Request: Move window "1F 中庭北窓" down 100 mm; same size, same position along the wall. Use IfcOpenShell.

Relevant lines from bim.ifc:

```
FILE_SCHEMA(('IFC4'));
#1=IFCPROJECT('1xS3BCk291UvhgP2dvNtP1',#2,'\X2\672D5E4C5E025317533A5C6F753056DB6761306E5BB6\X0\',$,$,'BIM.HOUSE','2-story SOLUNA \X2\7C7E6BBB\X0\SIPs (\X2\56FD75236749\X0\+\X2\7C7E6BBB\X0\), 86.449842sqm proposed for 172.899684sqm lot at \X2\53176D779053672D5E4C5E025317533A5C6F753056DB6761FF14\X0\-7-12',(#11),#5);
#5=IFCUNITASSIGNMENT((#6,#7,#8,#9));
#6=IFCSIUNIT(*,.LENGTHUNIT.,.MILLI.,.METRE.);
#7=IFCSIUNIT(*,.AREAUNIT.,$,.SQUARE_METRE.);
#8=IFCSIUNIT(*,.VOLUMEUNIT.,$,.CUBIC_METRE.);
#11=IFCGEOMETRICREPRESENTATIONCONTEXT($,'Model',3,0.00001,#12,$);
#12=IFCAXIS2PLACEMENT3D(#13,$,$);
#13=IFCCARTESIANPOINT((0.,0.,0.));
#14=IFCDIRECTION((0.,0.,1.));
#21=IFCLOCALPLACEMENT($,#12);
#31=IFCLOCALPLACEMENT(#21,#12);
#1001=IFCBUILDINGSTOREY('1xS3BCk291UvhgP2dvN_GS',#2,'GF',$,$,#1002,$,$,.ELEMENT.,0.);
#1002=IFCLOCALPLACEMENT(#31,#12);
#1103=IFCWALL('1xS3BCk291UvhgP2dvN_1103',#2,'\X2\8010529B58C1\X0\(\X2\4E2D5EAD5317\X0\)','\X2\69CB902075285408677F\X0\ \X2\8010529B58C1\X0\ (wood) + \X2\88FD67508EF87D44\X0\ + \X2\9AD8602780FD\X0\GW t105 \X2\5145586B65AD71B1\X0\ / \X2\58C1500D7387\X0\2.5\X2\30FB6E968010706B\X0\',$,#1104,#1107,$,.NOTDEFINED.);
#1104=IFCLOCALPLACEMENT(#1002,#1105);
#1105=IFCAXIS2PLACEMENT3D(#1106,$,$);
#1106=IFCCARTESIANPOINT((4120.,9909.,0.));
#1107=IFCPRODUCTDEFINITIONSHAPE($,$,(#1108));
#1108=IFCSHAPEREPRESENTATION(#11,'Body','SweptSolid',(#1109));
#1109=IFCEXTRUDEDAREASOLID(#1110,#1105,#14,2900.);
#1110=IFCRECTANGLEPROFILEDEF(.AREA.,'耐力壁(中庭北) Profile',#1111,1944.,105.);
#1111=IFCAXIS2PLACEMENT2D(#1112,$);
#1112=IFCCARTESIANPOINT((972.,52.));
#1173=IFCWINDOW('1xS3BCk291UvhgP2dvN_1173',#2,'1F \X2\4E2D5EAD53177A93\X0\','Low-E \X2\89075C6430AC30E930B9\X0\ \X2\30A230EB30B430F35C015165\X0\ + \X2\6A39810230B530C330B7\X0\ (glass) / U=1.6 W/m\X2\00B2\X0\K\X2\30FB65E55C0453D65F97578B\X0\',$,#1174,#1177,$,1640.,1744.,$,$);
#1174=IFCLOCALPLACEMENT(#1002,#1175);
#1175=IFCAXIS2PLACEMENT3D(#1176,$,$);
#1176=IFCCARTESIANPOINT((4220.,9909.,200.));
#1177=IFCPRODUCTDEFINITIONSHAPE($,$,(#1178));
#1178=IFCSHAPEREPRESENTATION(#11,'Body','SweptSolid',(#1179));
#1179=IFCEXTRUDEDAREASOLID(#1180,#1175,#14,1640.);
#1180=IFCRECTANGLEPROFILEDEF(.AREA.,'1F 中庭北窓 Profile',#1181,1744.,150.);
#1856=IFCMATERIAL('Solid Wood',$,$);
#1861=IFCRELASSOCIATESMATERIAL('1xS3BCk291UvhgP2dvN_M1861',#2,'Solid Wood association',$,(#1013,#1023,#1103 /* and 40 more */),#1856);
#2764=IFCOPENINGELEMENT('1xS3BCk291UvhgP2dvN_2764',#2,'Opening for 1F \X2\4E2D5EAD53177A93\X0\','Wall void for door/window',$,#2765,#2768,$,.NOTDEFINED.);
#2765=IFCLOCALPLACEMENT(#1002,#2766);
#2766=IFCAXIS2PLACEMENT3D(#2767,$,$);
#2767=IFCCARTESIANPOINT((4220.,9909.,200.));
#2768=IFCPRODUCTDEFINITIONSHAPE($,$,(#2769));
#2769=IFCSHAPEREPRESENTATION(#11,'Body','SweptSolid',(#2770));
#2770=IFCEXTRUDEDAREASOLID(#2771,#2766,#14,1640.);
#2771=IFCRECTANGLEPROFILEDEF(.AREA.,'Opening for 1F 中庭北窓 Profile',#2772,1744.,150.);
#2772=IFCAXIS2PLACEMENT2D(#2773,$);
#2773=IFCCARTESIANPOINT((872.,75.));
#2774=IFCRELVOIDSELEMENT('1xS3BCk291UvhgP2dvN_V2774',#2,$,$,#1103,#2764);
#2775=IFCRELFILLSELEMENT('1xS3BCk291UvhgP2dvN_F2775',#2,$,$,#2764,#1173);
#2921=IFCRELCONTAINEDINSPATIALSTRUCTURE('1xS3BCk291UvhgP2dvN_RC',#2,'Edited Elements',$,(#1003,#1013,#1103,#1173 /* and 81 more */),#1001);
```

```python
import numpy as np
import ifcopenshell
import ifcopenshell.api.geometry
import ifcopenshell.util.placement
import ifcopenshell.util.unit

model = ifcopenshell.open("bim.ifc")
unit_scale = ifcopenshell.util.unit.calculate_unit_scale(model)

window = model.by_guid("1xS3BCk291UvhgP2dvN_1173")
opening = window.FillsVoids[0].RelatingOpeningElement
dz = -100.0

shift = np.array([0.0, 0.0, dz])
# The window is not placed relative to its opening, so move both.
for product in (opening, window):
    matrix = ifcopenshell.util.placement.get_local_placement(product.ObjectPlacement)
    matrix[:3, 3] += shift
    ifcopenshell.api.geometry.edit_object_placement(model, product=product, matrix=matrix, is_si=False)

print(f"moved by {dz * unit_scale:+.3f} m")

model.write("bim_v2.ifc")
```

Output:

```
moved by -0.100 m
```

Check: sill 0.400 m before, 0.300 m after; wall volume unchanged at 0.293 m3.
